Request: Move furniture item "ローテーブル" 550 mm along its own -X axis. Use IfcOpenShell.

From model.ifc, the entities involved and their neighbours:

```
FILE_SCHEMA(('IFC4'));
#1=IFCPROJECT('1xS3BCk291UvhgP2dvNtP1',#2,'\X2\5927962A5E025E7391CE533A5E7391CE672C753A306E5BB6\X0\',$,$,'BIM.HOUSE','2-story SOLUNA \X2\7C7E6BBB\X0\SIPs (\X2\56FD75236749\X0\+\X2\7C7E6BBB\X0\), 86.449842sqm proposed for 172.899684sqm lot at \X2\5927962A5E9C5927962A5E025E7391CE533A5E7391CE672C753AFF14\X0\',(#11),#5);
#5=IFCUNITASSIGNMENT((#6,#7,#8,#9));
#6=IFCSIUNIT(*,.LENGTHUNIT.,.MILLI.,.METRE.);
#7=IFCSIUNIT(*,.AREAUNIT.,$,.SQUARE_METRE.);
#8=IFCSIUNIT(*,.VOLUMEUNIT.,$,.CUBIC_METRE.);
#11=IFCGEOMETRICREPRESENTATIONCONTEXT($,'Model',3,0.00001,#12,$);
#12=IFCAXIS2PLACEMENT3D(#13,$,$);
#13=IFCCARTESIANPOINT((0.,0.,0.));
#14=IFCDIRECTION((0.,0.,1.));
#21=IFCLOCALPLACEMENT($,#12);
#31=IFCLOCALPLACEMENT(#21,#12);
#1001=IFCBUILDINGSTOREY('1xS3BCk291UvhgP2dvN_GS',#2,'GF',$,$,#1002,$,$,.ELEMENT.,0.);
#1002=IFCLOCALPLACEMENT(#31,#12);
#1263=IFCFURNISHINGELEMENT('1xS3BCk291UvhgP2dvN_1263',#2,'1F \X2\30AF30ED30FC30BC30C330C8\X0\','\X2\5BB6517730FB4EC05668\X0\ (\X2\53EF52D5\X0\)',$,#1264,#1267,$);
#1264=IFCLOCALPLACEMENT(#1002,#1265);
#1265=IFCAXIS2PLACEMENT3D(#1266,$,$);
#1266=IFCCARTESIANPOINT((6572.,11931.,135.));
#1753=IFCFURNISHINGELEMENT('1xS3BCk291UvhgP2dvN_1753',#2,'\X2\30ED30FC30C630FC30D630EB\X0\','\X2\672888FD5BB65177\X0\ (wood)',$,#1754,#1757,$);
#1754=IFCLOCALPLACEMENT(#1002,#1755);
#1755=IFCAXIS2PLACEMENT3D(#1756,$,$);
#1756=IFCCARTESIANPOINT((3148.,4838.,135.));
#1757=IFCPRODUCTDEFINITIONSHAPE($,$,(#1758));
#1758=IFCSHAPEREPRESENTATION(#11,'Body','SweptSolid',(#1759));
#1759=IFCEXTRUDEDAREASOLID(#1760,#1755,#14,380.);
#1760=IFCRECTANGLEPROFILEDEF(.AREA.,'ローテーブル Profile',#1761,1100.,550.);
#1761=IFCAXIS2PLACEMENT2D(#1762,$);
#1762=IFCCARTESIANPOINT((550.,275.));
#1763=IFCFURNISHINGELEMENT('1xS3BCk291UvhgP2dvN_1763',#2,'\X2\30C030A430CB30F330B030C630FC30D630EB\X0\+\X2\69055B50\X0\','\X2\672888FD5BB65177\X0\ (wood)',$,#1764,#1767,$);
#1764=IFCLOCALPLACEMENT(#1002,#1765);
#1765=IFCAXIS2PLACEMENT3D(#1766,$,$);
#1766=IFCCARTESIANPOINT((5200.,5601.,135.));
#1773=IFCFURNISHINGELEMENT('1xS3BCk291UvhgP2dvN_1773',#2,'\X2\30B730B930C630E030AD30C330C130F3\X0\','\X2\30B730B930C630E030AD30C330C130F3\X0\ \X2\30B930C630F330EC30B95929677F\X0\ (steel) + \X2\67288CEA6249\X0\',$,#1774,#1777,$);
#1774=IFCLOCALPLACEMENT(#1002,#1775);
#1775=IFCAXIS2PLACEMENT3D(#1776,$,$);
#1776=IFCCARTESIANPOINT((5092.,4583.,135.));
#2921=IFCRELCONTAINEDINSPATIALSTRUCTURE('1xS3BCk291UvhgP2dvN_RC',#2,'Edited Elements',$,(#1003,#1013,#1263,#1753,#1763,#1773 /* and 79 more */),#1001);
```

```python
import ifcopenshell
import ifcopenshell.api.geometry
import ifcopenshell.util.placement
import ifcopenshell.util.unit

model = ifcopenshell.open("model.ifc")
unit_scale = ifcopenshell.util.unit.calculate_unit_scale(model)

item = model.by_guid("1xS3BCk291UvhgP2dvN_1753")
matrix = ifcopenshell.util.placement.get_local_placement(item.ObjectPlacement)
matrix[:3, 3] -= matrix[:3, 0] * 0.55 / unit_scale
ifcopenshell.api.geometry.edit_object_placement(model, product=item, matrix=matrix, is_si=False)

print(ifcopenshell.util.placement.get_local_placement(item.ObjectPlacement).round(3) + 0.0)

model.write("model_updated.ifc")
```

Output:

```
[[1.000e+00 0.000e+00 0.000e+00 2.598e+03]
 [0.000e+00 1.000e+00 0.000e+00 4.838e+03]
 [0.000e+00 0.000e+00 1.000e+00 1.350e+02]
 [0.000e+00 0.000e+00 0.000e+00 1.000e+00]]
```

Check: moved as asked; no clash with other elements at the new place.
